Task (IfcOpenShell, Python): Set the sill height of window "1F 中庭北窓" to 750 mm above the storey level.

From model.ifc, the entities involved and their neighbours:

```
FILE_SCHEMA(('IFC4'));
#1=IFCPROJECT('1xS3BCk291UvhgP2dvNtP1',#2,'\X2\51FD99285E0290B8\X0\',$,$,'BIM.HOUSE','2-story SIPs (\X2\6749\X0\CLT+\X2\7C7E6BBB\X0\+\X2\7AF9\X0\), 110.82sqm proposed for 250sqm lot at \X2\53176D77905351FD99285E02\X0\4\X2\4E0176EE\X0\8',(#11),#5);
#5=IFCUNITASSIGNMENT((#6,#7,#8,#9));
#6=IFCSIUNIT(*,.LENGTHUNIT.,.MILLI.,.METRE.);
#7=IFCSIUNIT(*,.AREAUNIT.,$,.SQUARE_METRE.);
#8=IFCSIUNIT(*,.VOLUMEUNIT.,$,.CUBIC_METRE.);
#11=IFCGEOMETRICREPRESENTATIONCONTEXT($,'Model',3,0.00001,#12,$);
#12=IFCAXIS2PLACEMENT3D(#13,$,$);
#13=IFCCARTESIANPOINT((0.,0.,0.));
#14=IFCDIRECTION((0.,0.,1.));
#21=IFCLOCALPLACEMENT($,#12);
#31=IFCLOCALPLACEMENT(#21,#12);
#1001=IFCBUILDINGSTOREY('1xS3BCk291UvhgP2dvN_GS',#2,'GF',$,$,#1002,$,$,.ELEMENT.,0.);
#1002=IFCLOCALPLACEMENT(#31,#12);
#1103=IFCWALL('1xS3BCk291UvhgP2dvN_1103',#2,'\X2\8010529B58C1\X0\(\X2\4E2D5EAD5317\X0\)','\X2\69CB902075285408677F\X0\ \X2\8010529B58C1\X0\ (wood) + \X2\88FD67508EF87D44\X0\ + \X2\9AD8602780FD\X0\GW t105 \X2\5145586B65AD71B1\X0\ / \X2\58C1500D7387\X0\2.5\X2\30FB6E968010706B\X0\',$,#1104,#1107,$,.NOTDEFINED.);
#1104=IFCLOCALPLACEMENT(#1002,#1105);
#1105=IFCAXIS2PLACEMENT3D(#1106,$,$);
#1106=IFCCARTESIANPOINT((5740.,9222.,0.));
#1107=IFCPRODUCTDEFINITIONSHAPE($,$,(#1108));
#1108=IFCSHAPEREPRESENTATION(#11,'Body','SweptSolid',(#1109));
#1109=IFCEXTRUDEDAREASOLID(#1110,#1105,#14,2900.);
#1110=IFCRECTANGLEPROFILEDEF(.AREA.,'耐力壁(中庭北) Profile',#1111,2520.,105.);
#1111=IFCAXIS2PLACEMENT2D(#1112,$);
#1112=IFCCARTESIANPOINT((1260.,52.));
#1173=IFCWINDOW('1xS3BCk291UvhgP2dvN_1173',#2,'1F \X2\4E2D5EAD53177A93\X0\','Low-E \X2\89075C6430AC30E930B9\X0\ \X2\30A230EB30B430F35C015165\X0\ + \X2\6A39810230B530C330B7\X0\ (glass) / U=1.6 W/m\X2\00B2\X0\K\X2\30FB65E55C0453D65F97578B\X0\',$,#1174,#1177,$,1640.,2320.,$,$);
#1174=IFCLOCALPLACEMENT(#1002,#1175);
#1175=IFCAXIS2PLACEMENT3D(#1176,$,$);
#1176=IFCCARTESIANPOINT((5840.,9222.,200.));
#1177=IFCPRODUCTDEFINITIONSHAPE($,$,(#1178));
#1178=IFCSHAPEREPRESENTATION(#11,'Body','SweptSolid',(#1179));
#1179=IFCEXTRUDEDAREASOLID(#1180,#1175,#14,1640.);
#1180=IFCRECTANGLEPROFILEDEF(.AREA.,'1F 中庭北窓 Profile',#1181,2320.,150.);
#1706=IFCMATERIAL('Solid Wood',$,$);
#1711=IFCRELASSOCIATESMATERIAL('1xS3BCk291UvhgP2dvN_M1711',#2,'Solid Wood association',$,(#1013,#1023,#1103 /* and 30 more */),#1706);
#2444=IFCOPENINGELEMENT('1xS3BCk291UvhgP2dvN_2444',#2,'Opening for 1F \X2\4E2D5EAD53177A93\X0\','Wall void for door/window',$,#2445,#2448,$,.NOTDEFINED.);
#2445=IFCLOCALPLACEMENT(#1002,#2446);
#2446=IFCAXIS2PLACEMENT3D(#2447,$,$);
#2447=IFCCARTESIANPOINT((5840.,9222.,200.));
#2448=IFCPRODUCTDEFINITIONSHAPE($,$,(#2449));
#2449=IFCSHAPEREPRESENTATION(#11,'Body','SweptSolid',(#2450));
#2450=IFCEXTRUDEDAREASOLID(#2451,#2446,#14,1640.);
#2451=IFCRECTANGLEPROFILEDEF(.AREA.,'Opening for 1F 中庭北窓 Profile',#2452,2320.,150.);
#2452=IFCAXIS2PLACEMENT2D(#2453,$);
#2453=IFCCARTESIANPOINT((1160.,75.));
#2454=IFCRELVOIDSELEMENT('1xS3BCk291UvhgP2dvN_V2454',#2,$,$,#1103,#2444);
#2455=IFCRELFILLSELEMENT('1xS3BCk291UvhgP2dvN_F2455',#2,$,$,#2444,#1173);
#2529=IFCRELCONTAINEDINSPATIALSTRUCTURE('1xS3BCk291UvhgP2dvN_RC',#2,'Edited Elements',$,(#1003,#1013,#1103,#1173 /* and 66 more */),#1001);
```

```python
import numpy as np
import ifcopenshell
import ifcopenshell.api.geometry
import ifcopenshell.geom
import ifcopenshell.util.element
import ifcopenshell.util.placement
import ifcopenshell.util.shape
import ifcopenshell.util.unit

model = ifcopenshell.open("model.ifc")
unit_scale = ifcopenshell.util.unit.calculate_unit_scale(model)

window = model.by_guid("1xS3BCk291UvhgP2dvN_1173")
opening = window.FillsVoids[0].RelatingOpeningElement
storey = ifcopenshell.util.element.get_container(window, ifc_class="IfcBuildingStorey")
level = ifcopenshell.util.placement.get_local_placement(storey.ObjectPlacement)[2, 3]

# The opening's origin need not be at the sill, so measure its lowest point.
shape = ifcopenshell.geom.create_shape(ifcopenshell.geom.settings(), opening)
bottom = ifcopenshell.util.shape.get_shape_bottom_elevation(shape, shape.geometry) / unit_scale
dz = level + 0.75 / unit_scale - bottom

shift = np.array([0.0, 0.0, dz])
# The window is not placed relative to its opening, so move both.
for product in (opening, window):
    matrix = ifcopenshell.util.placement.get_local_placement(product.ObjectPlacement)
    matrix[:3, 3] += shift
    ifcopenshell.api.geometry.edit_object_placement(model, product=product, matrix=matrix, is_si=False)

print(f"moved by {dz * unit_scale:+.3f} m")

model.write("model_v2.ifc")
```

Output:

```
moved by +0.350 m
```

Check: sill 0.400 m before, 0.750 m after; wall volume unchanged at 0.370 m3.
